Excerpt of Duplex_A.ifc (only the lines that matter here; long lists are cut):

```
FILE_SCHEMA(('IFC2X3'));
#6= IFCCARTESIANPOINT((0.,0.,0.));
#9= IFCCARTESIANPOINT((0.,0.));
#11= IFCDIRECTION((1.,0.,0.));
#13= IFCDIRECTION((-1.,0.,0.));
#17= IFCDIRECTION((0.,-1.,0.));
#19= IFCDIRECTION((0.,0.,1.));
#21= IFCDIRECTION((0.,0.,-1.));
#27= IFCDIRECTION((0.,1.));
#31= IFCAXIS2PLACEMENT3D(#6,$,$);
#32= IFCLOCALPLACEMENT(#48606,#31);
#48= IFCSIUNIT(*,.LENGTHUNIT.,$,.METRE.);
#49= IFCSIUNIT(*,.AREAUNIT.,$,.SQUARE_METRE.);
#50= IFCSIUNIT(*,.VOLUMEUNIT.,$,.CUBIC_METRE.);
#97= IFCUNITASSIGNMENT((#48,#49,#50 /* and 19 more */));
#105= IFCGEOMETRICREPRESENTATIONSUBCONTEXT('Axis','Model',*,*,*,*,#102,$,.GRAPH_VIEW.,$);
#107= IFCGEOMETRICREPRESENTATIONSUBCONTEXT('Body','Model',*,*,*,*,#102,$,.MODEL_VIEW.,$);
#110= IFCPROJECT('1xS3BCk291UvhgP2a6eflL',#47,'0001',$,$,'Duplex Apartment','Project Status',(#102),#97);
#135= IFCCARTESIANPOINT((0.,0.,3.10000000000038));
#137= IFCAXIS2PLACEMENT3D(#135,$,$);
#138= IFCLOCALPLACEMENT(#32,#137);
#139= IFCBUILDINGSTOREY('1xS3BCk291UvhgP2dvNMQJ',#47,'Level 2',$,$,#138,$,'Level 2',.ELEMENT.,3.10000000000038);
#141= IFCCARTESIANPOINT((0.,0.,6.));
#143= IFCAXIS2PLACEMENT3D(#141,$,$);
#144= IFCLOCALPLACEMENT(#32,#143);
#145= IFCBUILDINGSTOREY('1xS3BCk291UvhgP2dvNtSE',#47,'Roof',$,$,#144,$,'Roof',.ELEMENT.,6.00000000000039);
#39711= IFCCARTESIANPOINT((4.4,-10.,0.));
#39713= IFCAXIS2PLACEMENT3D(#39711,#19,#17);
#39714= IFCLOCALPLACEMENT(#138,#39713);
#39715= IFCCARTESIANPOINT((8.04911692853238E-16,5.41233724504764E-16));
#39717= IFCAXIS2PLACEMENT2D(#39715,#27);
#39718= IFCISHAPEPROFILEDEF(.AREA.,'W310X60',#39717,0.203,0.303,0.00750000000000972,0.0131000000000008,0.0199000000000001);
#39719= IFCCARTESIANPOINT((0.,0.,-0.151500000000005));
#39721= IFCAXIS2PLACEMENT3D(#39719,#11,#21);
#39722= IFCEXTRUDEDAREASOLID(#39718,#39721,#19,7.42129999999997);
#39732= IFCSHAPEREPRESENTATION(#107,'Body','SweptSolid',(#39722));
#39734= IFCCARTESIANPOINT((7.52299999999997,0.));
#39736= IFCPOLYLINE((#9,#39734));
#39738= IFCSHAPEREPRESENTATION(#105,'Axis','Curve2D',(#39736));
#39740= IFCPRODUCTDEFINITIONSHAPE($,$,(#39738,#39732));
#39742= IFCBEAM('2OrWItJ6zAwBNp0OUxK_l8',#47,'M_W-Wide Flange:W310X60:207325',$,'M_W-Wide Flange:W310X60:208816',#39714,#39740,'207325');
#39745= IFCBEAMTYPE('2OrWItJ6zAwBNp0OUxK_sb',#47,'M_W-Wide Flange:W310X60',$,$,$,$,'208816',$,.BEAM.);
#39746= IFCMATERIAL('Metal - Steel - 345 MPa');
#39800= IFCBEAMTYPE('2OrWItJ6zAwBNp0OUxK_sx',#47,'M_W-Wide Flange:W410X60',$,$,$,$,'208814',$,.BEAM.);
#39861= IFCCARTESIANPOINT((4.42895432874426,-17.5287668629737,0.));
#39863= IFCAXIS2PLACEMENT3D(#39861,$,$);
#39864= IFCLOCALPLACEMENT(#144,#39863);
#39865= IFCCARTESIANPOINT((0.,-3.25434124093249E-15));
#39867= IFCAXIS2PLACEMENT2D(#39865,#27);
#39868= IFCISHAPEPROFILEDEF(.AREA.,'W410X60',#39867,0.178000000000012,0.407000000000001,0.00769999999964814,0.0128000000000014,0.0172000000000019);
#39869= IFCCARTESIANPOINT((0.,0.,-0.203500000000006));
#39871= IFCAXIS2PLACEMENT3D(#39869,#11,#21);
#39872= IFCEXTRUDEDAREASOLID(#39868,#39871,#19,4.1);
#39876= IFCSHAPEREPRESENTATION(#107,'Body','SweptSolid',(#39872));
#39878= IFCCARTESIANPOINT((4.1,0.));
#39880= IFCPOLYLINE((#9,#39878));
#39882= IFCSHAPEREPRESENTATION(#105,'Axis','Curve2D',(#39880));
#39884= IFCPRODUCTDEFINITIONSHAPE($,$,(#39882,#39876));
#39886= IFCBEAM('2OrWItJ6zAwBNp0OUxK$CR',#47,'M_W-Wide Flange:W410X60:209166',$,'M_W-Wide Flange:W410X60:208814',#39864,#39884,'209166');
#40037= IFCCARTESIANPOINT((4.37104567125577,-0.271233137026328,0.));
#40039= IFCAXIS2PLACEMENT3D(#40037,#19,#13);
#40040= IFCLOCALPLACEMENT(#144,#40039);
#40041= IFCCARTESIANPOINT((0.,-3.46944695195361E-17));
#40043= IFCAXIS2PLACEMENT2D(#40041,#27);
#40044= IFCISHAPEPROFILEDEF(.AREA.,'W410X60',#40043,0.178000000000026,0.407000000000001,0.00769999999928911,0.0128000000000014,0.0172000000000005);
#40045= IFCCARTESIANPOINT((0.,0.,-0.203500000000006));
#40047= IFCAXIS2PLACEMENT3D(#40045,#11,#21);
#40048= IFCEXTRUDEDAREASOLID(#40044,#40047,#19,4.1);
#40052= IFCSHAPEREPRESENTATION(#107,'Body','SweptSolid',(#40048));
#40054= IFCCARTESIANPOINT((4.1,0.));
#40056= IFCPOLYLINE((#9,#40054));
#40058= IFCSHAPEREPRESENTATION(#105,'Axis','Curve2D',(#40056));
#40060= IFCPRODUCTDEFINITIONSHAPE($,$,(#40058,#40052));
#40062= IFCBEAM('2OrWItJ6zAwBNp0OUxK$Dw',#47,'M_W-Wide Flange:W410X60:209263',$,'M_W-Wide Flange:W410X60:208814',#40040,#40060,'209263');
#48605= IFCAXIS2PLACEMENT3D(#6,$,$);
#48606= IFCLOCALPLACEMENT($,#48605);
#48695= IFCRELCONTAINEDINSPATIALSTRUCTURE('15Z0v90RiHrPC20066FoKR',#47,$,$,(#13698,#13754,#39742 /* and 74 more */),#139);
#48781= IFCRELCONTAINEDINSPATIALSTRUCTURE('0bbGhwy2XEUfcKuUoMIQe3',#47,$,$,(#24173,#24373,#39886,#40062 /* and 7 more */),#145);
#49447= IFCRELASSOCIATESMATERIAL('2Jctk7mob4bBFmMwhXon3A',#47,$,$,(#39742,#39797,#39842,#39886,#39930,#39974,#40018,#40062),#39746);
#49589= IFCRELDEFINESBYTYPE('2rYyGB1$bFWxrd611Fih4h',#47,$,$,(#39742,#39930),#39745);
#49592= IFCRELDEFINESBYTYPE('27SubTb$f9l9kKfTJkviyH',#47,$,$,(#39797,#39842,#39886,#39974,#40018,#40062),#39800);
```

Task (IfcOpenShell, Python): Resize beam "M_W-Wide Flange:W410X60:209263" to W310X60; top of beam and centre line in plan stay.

```python
import ifcopenshell
import ifcopenshell.api.type
import ifcopenshell.util.element
import ifcopenshell.util.representation

model = ifcopenshell.open("Duplex_A.ifc")

member = model.by_guid("2OrWItJ6zAwBNp0OUxK$Dw")
source = next(p for p in model.by_type("IfcIShapeProfileDef") if p.ProfileName == "W310X60")

body = ifcopenshell.util.representation.get_representation(member, "Model", "Body")
solid = body.Items[0]
old_profile = solid.SweptArea

# Copy the section's sizes but keep this member's own profile position.
profile = ifcopenshell.util.element.copy(model, source)
# Profiles are centred, so shift by half the change in depth to hold the top.
shift = (old_profile.OverallDepth - profile.OverallDepth) / 2
x, y = old_profile.Position.Location.Coordinates
up = (-1.0, 0.0)  # upwards, in the solid's own plane
location = model.createIfcCartesianPoint((x + up[0] * shift, y + up[1] * shift))
profile.Position = model.createIfcAxis2Placement2D(location, old_profile.Position.RefDirection)
solid.SweptArea = profile
if not model.get_total_inverses(old_profile):
    ifcopenshell.util.element.remove_deep2(model, old_profile)

new_type = model.by_guid("2OrWItJ6zAwBNp0OUxK_sb")
ifcopenshell.api.type.assign_type(
    model, related_objects=[member], relating_type=new_type, should_map_representations=False
)
member.Name = member.Name.replace("W410X60", "W310X60")
member.ObjectType = "M_W-Wide Flange:W310X60:208814"

print(solid.SweptArea)

model.write("Duplex_A_v2.ifc")
```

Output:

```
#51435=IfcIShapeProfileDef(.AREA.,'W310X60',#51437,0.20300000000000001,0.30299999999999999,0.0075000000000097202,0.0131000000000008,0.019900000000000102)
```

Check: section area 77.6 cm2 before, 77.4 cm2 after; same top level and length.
